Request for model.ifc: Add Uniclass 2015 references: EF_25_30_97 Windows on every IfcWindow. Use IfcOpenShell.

First a look at what the model holds.

```python
import ifcopenshell

model = ifcopenshell.open("model.ifc")
print(model.schema)
print("classifications:", [c.Name for c in model.by_type("IfcClassification")])
for ifc_class in ("IfcDoor", "IfcRoof", "IfcStair", "IfcWall", "IfcWindow"):
    print(ifc_class, len(model.by_type(ifc_class)))
```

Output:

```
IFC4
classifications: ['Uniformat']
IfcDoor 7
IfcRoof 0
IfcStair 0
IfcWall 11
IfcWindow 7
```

```python
import ifcopenshell
import ifcopenshell.api.classification

model = ifcopenshell.open("model.ifc")

system = ifcopenshell.api.classification.add_classification(model, classification="Uniclass 2015")

codes = {
    "IfcWindow": ("EF_25_30_97", "Windows"),
}
for ifc_class, (code, name) in codes.items():
    products = model.by_type(ifc_class)
    ifcopenshell.api.classification.add_reference(
        model, products=products, classification=system, identification=code, name=name
    )
    print(code, len(products))

model.write("model-out.ifc")
```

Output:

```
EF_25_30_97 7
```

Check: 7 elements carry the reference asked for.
